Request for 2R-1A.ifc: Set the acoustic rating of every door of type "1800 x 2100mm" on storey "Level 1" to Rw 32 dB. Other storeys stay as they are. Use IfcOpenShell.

First a look at what the model holds.

```python
import ifcopenshell
import ifcopenshell.util.element

model = ifcopenshell.open("2R-1A.ifc")
print(model.schema)
storey = next(s for s in model.by_type("IfcBuildingStorey") if s.Name == "Level 1")
doors = [e for e in ifcopenshell.util.element.get_decomposition(storey) if e.is_a("IfcDoor")]
seen = {}
for e in doors:
    element_type = ifcopenshell.util.element.get_type(e)
    key = (element_type.Name if element_type != e and element_type else None, ifcopenshell.util.element.get_pset(e, "Pset_DoorCommon", "AcousticRating"))
    seen[key] = seen.get(key, 0) + 1
for (name, value), count in sorted(seen.items(), key=str):
    print(count, "x", name, "|", value)
```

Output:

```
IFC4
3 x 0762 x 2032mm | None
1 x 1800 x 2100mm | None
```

```python
import ifcopenshell
import ifcopenshell.api.pset
import ifcopenshell.util.element

model = ifcopenshell.open("2R-1A.ifc")

storey = next(s for s in model.by_type("IfcBuildingStorey") if s.Name == "Level 1")
doors = [e for e in ifcopenshell.util.element.get_decomposition(storey) if e.is_a("IfcDoor")]

count = 0
for e in doors:
    element_type = ifcopenshell.util.element.get_type(e)
    if element_type in (None, e) or element_type.Name != "1800 x 2100mm":
        continue
    # add_pset returns the element's existing set when there is one.
    pset = ifcopenshell.api.pset.add_pset(model, product=e, name="Pset_DoorCommon")
    ifcopenshell.api.pset.edit_pset(model, pset=pset, properties={"AcousticRating": "Rw 32 dB"})
    count += 1

print(count, "doors updated")

model.write("2R-1A_v2.ifc")
```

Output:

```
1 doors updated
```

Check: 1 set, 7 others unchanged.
